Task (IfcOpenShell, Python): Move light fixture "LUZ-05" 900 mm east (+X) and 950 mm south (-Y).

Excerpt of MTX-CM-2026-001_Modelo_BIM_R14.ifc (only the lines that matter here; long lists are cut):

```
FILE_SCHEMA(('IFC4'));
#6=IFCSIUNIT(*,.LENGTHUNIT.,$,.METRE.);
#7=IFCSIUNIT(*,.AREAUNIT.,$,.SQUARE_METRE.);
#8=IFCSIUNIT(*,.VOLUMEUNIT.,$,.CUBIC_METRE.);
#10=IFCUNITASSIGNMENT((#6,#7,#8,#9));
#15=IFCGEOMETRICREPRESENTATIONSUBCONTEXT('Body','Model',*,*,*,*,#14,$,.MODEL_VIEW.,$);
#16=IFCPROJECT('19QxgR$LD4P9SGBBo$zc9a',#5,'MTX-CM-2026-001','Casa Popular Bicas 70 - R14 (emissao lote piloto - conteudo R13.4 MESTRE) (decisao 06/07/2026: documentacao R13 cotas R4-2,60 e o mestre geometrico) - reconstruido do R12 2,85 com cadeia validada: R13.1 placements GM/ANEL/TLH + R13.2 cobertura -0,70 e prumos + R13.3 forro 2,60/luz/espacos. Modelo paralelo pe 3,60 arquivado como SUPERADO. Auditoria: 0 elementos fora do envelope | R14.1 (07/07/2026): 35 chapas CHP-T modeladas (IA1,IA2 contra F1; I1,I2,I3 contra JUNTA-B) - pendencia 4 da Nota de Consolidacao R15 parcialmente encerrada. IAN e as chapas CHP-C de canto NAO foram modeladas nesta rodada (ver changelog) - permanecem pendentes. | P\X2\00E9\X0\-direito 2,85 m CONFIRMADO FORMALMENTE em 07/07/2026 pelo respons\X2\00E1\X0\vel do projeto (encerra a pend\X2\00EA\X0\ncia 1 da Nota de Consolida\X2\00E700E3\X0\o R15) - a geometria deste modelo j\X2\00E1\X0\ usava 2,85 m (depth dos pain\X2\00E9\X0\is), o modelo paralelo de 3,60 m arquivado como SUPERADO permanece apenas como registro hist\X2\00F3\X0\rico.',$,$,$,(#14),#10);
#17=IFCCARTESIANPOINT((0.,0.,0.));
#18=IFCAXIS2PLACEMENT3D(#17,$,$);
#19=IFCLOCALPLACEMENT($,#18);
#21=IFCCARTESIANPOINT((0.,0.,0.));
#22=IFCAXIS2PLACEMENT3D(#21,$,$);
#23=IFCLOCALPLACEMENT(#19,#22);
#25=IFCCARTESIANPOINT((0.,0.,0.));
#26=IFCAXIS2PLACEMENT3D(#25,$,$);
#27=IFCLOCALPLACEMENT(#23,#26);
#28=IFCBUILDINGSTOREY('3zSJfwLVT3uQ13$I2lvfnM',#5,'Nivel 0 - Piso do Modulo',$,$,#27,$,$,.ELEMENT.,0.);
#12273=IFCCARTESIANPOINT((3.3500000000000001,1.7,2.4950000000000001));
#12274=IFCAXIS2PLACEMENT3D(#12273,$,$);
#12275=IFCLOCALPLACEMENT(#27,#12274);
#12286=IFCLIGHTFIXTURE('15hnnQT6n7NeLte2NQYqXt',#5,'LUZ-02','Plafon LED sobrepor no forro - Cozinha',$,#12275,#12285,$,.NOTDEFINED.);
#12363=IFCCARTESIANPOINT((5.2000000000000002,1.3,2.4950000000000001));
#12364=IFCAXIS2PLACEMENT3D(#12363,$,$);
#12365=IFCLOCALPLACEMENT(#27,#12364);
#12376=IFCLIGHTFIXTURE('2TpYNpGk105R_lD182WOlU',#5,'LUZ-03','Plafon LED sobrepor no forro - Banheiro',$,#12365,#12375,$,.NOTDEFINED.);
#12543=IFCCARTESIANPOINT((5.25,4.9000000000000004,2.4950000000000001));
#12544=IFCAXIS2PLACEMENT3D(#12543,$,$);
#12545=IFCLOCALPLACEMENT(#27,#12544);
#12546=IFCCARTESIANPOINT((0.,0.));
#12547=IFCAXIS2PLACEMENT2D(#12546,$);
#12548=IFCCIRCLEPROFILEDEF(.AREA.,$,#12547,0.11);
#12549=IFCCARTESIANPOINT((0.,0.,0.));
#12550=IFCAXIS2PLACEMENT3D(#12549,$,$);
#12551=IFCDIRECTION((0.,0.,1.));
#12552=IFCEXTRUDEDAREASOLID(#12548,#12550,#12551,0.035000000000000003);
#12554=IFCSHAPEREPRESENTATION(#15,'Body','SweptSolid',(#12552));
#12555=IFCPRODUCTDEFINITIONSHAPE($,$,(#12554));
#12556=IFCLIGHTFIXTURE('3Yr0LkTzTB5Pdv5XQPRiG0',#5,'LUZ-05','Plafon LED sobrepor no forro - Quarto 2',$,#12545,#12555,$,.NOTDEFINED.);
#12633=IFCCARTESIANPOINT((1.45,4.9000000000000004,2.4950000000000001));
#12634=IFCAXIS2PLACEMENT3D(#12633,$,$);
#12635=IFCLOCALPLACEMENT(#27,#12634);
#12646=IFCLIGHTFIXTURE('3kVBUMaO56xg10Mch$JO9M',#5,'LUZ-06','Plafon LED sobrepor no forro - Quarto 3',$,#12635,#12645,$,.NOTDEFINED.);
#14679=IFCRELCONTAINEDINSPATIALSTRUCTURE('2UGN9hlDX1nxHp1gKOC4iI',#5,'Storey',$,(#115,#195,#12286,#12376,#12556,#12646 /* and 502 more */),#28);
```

```python
import ifcopenshell
import ifcopenshell.api.geometry
import ifcopenshell.util.placement

model = ifcopenshell.open("MTX-CM-2026-001_Modelo_BIM_R14.ifc")

item = model.by_guid("3Yr0LkTzTB5Pdv5XQPRiG0")
matrix = ifcopenshell.util.placement.get_local_placement(item.ObjectPlacement)
matrix[0, 3] += 0.9
matrix[1, 3] -= 0.95
ifcopenshell.api.geometry.edit_object_placement(model, product=item, matrix=matrix, is_si=False)

print(ifcopenshell.util.placement.get_local_placement(item.ObjectPlacement).round(3) + 0.0)

model.write("MTX-CM-2026-001_Modelo_BIM_R14_rev.ifc")
```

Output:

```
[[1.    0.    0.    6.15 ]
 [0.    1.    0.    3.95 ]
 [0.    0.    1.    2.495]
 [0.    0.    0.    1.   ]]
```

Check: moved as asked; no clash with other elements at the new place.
